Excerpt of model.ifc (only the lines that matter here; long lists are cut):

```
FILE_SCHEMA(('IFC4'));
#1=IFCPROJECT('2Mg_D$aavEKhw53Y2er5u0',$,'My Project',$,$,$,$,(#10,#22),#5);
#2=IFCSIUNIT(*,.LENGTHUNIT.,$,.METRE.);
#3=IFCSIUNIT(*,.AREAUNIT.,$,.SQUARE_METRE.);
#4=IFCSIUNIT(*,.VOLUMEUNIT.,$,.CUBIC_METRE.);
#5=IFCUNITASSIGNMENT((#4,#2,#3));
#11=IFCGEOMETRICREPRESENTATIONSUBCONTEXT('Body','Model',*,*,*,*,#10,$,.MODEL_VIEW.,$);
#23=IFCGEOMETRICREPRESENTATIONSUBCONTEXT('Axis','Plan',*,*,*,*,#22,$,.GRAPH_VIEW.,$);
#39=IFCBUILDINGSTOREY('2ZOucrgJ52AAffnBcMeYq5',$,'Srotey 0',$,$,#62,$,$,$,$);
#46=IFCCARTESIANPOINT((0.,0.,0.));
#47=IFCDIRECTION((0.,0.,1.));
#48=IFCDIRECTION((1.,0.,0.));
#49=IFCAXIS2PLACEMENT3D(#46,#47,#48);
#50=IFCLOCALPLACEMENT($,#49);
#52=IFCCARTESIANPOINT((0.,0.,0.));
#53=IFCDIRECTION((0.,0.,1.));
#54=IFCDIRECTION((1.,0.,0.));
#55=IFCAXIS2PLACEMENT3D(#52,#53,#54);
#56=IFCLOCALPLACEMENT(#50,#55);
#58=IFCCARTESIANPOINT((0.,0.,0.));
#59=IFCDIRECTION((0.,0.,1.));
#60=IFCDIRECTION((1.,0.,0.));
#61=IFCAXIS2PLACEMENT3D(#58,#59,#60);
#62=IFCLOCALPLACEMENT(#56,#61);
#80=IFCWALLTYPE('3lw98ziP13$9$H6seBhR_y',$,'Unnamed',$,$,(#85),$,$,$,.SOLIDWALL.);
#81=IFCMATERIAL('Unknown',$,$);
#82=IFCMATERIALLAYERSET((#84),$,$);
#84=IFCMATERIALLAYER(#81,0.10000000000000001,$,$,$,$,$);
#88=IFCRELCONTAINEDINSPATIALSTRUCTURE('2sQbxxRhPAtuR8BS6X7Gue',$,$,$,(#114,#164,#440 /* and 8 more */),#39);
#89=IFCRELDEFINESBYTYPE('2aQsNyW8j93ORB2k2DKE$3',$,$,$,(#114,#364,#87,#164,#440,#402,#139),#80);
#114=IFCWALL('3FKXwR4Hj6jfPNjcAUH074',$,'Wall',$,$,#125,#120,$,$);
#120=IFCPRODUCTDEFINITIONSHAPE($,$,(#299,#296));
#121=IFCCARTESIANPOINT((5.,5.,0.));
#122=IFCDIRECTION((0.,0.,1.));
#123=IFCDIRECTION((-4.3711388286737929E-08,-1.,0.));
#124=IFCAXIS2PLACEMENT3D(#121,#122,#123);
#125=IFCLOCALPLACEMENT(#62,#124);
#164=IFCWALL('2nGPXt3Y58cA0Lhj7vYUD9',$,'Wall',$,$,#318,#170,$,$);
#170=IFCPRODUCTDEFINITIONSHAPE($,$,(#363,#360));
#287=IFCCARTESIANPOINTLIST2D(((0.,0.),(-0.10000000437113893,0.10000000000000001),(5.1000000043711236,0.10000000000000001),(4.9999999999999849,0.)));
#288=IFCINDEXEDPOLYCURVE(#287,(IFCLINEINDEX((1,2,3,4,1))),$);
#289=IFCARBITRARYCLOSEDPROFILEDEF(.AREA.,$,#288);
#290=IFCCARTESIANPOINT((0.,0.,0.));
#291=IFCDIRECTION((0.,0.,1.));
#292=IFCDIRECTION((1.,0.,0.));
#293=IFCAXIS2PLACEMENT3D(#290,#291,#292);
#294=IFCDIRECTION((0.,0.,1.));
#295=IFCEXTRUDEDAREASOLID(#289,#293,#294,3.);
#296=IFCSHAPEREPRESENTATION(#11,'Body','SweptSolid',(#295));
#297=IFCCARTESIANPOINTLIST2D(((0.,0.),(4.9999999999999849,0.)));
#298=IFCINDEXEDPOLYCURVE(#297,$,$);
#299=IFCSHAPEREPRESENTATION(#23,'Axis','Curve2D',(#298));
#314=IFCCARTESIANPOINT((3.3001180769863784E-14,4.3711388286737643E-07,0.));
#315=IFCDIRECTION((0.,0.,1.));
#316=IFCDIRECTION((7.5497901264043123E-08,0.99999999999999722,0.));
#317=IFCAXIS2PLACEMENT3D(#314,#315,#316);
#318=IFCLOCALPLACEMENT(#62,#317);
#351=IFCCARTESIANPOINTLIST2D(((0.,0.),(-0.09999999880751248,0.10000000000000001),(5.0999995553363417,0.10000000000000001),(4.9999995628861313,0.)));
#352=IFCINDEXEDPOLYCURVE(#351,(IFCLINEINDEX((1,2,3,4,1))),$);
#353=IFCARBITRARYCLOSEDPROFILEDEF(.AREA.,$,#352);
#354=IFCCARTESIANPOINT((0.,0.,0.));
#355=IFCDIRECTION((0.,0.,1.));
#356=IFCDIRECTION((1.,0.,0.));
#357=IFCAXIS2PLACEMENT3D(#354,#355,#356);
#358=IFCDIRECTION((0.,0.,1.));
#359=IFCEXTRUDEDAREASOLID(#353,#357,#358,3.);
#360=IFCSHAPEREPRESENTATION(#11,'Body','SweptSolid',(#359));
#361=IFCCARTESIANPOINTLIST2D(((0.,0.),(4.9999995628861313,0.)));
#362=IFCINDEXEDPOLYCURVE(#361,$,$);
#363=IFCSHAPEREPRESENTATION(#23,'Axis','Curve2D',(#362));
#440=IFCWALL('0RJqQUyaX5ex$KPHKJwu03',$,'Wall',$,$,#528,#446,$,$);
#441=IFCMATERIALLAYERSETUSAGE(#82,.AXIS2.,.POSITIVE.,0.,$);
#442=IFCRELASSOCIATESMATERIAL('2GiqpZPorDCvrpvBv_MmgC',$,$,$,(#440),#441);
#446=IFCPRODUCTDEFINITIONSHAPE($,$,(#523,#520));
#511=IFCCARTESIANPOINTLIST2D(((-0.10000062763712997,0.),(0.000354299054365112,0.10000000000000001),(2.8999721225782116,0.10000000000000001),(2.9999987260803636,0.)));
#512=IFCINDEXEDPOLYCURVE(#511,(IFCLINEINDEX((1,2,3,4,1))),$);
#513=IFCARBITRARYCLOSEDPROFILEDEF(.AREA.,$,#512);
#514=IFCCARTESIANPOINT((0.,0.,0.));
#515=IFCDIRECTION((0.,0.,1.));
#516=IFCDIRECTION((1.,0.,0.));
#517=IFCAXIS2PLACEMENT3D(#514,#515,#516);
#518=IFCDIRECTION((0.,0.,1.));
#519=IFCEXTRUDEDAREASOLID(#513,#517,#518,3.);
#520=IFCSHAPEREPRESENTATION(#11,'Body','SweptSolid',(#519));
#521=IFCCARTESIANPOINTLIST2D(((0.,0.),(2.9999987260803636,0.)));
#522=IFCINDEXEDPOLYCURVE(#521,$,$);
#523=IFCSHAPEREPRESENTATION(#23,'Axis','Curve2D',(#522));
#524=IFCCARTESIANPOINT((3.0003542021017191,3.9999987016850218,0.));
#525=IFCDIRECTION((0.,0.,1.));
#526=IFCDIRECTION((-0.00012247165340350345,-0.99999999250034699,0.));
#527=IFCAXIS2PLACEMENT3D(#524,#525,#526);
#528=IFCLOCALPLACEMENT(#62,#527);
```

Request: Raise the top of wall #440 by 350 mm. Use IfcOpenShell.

```python
import ifcopenshell
import ifcopenshell.geom
import ifcopenshell.util.representation
import ifcopenshell.util.shape

model = ifcopenshell.open("model.ifc")
settings = ifcopenshell.geom.settings()


def volume(element):
    """Net volume in cubic metres, openings subtracted."""
    shape = ifcopenshell.geom.create_shape(settings, element)
    return ifcopenshell.util.shape.get_volume(shape.geometry)


wall = model.by_guid("0RJqQUyaX5ex$KPHKJwu03")
before = volume(wall)

body = ifcopenshell.util.representation.get_representation(wall, "Model", "Body")
solid = body.Items[0]
old_height = solid.Depth
solid.Depth += 0.35
after = volume(wall)

print(f"height {old_height:g} -> {solid.Depth:g}, volume {before:.3f} -> {after:.3f} m3")

model.write("model_edited.ifc")
```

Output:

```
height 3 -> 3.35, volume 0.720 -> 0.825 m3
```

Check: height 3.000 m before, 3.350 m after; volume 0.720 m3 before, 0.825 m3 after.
